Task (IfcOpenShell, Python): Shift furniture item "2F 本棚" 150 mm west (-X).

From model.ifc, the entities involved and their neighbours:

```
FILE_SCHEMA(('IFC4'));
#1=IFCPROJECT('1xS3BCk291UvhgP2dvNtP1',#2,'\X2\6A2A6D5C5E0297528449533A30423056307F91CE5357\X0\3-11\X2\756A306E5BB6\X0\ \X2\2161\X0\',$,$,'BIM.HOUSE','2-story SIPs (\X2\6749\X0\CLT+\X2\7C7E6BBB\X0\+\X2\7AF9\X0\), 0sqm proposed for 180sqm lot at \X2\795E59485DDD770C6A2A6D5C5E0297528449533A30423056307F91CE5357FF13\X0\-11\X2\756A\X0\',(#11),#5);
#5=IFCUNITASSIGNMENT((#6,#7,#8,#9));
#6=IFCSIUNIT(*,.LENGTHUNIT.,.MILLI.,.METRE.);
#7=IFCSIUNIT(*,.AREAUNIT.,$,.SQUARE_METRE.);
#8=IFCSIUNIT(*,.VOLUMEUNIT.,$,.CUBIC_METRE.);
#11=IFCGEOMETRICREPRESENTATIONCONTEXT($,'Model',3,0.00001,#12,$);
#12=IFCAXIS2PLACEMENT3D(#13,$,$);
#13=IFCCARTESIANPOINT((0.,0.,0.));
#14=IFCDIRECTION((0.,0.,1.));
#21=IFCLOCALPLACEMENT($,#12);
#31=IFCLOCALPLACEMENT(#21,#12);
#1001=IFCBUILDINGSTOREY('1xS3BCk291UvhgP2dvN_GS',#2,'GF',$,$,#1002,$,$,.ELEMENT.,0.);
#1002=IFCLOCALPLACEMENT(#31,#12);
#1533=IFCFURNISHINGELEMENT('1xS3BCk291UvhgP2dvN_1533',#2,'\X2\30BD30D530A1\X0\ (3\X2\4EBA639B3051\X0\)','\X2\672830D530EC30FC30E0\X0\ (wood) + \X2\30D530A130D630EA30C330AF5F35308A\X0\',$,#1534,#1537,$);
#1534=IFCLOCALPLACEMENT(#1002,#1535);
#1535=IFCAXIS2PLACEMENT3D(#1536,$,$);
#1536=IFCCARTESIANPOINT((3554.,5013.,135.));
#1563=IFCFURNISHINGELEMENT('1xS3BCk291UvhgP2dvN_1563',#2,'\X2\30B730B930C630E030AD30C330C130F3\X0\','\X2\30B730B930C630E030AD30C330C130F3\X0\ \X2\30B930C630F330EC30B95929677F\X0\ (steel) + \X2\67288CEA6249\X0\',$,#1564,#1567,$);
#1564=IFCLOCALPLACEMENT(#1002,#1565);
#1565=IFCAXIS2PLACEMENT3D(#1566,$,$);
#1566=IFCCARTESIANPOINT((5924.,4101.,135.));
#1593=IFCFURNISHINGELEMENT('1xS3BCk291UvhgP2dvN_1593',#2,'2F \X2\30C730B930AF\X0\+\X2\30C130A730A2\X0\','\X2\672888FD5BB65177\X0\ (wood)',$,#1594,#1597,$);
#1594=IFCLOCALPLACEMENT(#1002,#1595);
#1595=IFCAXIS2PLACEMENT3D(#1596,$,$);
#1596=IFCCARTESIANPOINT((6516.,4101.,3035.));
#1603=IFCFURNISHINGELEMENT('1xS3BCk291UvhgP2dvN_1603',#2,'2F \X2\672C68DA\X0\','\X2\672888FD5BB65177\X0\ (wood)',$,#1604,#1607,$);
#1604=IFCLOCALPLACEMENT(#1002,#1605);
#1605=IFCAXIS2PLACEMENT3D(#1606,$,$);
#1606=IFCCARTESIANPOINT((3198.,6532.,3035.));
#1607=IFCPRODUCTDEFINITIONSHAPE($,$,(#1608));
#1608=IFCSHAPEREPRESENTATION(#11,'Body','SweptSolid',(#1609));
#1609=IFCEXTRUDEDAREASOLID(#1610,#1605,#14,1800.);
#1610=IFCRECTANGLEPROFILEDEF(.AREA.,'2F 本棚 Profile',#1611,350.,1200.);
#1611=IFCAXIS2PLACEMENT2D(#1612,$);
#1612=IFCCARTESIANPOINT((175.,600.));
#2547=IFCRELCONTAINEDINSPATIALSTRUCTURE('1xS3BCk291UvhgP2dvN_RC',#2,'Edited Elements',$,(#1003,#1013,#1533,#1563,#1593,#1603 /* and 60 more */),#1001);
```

```python
import ifcopenshell
import ifcopenshell.api.geometry
import ifcopenshell.util.placement
import ifcopenshell.util.unit

model = ifcopenshell.open("model.ifc")
unit_scale = ifcopenshell.util.unit.calculate_unit_scale(model)

item = model.by_guid("1xS3BCk291UvhgP2dvN_1603")
matrix = ifcopenshell.util.placement.get_local_placement(item.ObjectPlacement)
matrix[0, 3] -= 0.15 / unit_scale
ifcopenshell.api.geometry.edit_object_placement(model, product=item, matrix=matrix, is_si=False)

print(ifcopenshell.util.placement.get_local_placement(item.ObjectPlacement).round(3) + 0.0)

model.write("model_v2.ifc")
```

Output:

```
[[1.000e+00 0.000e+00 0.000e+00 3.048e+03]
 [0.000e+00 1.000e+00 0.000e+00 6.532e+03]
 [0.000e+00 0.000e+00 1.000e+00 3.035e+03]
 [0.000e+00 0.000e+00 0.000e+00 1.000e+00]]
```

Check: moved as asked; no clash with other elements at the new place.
